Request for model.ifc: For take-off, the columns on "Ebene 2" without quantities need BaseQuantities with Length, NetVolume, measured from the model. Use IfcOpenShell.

First a look at what the model holds.

```python
import ifcopenshell
import ifcopenshell.util.element
import ifcopenshell.util.unit

model = ifcopenshell.open("model.ifc")
print(model.schema)
for unit_type in ("LENGTHUNIT", "AREAUNIT", "VOLUMEUNIT"):
    print(unit_type, ifcopenshell.util.unit.calculate_unit_scale(model, unit_type))
storey = next(s for s in model.by_type("IfcBuildingStorey") if s.Name == "Ebene 2")
columns = [e for e in ifcopenshell.util.element.get_decomposition(storey) if e.is_a("IfcColumn")]
for e in sorted(columns, key=lambda e: e.id()):
    print(e.id(), e.is_a(), e.Name, list(ifcopenshell.util.element.get_psets(e, qtos_only=True)), sep=" | ")
```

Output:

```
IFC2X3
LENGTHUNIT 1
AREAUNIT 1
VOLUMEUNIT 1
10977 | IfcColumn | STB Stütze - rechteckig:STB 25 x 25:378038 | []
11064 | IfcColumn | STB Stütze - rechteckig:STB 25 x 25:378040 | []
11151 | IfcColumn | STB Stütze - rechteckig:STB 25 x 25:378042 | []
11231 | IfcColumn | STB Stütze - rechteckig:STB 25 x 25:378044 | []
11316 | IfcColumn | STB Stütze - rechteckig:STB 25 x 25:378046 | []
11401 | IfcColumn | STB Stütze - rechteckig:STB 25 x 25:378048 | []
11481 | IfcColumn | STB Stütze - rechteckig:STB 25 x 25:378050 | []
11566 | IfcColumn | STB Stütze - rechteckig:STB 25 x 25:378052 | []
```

```python
import ifcopenshell
import ifcopenshell.api.pset
import ifcopenshell.geom
import ifcopenshell.util.element
import ifcopenshell.util.shape
import ifcopenshell.util.unit

model = ifcopenshell.open("model.ifc")
unit_scale = ifcopenshell.util.unit.calculate_unit_scale(model)
volume_scale = ifcopenshell.util.unit.calculate_unit_scale(model, "VOLUMEUNIT")
settings = ifcopenshell.geom.settings()

storey = next(s for s in model.by_type("IfcBuildingStorey") if s.Name == "Ebene 2")
columns = [e for e in ifcopenshell.util.element.get_decomposition(storey) if e.is_a("IfcColumn")]

for e in sorted(columns, key=lambda e: e.id()):
    if ifcopenshell.util.element.get_psets(e, qtos_only=True, should_inherit=False):
        continue
    # Geometry comes back in metres, in the element's own axes.
    shape = ifcopenshell.geom.create_shape(settings, e)
    values = {
        "Length": ifcopenshell.util.shape.get_z(shape.geometry) / unit_scale,
        "NetVolume": ifcopenshell.util.shape.get_volume(shape.geometry) / volume_scale,
    }
    qto = ifcopenshell.api.pset.add_qto(model, product=e, name="BaseQuantities")
    ifcopenshell.api.pset.edit_qto(model, qto=qto, properties=values)
    print(e.id(), {k: round(v, 3) for k, v in values.items()})

model.write("model_rev.ifc")
```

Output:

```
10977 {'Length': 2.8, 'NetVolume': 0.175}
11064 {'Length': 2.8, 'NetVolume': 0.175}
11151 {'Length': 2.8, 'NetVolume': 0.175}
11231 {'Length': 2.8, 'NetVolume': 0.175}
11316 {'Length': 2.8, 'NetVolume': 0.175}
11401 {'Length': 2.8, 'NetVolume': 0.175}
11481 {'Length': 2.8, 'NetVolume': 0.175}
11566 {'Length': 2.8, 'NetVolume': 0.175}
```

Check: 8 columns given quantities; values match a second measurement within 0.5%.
